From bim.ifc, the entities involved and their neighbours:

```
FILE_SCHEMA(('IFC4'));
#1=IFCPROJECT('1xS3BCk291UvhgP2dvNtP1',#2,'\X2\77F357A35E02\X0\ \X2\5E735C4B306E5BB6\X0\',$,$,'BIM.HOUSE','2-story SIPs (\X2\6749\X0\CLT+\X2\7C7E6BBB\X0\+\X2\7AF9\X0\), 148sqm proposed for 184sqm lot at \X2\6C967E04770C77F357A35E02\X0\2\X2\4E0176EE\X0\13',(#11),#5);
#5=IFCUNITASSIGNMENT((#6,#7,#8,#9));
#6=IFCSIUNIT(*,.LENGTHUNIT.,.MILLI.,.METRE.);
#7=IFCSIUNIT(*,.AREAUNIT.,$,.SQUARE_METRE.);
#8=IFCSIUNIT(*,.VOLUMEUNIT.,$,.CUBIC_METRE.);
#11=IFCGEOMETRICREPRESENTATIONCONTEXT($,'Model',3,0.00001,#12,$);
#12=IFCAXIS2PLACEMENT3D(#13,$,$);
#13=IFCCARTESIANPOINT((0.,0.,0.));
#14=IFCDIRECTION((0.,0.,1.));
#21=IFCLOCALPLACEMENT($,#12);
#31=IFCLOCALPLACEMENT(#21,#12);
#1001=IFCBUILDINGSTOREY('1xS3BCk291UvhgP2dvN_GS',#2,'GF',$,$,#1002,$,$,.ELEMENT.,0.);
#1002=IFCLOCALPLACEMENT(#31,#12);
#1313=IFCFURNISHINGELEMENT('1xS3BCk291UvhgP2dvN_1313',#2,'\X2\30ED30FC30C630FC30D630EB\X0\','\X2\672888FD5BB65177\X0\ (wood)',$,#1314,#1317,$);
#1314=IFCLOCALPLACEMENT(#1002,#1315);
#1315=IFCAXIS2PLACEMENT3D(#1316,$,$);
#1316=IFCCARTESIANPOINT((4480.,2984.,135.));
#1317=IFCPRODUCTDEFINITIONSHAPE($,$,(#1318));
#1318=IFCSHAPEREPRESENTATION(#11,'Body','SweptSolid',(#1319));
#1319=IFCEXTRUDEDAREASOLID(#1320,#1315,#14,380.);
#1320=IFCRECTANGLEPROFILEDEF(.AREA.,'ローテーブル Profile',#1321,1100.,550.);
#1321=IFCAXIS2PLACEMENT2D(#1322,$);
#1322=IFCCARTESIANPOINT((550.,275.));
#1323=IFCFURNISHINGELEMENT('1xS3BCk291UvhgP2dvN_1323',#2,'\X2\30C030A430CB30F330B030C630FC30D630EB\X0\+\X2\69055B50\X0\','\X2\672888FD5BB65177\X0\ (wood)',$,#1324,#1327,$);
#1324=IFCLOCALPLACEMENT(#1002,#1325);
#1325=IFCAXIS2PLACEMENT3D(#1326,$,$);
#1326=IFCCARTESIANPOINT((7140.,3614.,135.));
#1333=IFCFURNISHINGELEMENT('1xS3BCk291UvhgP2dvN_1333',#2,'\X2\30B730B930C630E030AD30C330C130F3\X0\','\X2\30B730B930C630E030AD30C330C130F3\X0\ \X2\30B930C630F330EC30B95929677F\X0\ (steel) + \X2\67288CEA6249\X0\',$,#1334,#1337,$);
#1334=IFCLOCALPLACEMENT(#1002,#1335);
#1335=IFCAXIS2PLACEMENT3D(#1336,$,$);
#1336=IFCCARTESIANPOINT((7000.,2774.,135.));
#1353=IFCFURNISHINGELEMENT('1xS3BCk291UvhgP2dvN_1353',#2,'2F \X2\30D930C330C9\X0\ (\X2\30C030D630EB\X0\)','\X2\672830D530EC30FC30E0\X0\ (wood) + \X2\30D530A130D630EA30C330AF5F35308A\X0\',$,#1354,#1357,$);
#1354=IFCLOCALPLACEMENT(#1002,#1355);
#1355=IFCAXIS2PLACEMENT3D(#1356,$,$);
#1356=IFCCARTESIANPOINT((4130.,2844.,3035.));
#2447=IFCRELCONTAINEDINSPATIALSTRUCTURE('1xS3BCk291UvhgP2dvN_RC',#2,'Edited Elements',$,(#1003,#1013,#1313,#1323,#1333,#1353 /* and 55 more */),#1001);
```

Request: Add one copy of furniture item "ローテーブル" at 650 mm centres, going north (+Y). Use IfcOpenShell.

```python
import numpy as np
import ifcopenshell
import ifcopenshell.api.geometry
import ifcopenshell.api.root
import ifcopenshell.util.element
import ifcopenshell.util.placement
import ifcopenshell.util.unit

model = ifcopenshell.open("bim.ifc")
unit_scale = ifcopenshell.util.unit.calculate_unit_scale(model)


def reuse_history(source, copy):
    """copy_class also copies each property set's owner history, people and application; keep the originals."""
    for rel in copy.IsDefinedBy:
        if rel.is_a("IfcRelDefinesByProperties") and (history := rel.RelatingPropertyDefinition.OwnerHistory):
            rel.RelatingPropertyDefinition.OwnerHistory = source.OwnerHistory
            ifcopenshell.util.element.remove_deep2(model, history)


source = model.by_guid("1xS3BCk291UvhgP2dvN_1313")
base = ifcopenshell.util.placement.get_local_placement(source.ObjectPlacement)
step = np.array([0.0, 1.0, 0.0]) * 0.65 / unit_scale

for i in range(1, 2):
    copy = ifcopenshell.api.root.copy_class(model, product=source)
    copy.Representation = ifcopenshell.util.element.copy_deep(
        model, source.Representation, exclude=["IfcGeometricRepresentationContext", "IfcRepresentationMap"]
    )
    reuse_history(source, copy)
    matrix = base.copy()
    matrix[:3, 3] += i * step
    print("added at", matrix[:3, 3].round(3) + 0.0)
    ifcopenshell.api.geometry.edit_object_placement(model, product=copy, matrix=matrix, is_si=False)

model.write("bim_v2.ifc")
```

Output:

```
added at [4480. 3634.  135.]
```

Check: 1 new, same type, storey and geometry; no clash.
